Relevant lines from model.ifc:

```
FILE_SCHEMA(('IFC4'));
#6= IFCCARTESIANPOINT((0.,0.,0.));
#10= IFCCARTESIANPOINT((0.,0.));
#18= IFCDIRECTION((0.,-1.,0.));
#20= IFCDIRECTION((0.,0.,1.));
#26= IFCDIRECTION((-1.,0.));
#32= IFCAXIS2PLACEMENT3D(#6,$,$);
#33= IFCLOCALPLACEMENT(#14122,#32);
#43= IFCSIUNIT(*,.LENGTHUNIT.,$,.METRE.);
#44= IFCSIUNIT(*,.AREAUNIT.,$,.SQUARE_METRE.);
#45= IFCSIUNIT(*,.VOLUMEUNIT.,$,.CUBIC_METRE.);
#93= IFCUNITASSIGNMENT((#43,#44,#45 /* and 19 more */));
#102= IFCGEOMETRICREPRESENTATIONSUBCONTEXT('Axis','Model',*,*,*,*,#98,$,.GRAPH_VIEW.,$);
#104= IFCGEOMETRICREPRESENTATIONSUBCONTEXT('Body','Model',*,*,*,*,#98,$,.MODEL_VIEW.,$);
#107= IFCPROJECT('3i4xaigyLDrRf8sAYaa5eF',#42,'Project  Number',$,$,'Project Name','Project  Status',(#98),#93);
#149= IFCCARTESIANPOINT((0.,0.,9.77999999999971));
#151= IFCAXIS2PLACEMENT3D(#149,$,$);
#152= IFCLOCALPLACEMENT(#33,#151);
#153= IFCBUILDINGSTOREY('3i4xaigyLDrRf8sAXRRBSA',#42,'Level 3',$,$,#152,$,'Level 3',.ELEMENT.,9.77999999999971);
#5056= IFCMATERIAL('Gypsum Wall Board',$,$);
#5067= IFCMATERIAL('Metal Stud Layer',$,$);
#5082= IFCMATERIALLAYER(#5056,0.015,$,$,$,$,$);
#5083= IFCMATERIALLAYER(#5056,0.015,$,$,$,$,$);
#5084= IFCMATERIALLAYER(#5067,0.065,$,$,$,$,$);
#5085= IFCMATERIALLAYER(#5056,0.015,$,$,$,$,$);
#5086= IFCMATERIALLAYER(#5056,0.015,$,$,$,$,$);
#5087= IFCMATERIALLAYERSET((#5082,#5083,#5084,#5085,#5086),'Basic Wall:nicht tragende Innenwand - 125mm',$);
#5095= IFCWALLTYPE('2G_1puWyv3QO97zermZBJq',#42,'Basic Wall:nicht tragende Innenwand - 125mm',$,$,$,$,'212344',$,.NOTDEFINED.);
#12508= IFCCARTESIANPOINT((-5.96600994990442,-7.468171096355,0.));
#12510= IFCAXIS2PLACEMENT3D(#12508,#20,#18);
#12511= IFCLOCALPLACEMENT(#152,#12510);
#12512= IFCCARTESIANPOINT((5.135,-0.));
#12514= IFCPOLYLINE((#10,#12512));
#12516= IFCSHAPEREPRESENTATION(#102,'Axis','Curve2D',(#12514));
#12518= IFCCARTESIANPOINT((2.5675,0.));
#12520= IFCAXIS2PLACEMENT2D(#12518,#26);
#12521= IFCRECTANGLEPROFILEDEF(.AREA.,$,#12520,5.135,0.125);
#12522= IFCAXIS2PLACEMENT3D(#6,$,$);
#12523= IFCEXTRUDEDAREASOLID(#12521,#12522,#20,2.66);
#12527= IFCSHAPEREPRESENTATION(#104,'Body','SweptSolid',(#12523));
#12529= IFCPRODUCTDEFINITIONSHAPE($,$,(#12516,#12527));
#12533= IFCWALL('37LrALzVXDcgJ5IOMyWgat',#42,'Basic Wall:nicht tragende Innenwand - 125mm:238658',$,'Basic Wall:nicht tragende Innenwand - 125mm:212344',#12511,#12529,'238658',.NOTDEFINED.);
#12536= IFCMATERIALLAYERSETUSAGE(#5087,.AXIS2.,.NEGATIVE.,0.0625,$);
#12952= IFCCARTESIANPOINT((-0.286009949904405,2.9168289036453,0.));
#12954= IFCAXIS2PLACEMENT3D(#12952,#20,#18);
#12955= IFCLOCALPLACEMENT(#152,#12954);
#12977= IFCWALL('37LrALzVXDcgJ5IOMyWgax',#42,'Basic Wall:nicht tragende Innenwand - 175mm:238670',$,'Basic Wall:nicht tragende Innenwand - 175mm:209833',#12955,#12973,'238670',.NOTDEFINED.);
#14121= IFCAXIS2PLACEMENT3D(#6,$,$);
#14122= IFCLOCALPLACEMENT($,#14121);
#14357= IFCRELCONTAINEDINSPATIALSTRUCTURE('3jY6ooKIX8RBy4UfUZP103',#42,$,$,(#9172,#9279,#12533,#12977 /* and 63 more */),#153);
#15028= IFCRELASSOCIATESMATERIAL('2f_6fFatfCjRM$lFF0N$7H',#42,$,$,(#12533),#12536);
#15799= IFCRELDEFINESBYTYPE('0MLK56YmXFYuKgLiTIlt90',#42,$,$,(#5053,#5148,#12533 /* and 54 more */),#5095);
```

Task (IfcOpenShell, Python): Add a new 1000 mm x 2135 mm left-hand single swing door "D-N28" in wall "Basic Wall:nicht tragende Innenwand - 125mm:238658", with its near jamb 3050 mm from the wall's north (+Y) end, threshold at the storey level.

```python
import numpy as np
import ifcopenshell
import ifcopenshell.api.feature
import ifcopenshell.api.geometry
import ifcopenshell.api.root
import ifcopenshell.api.spatial
import ifcopenshell.geom
import ifcopenshell.util.element
import ifcopenshell.util.placement
import ifcopenshell.util.representation
import ifcopenshell.util.shape
import ifcopenshell.util.unit

model = ifcopenshell.open("model.ifc")
unit_scale = ifcopenshell.util.unit.calculate_unit_scale(model)
settings = ifcopenshell.geom.settings()


def volume(element):
    """Net volume in cubic metres, openings subtracted."""
    shape = ifcopenshell.geom.create_shape(settings, element)
    return ifcopenshell.util.shape.get_volume(shape.geometry)


wall = model.by_id(12533)
storey = ifcopenshell.util.element.get_container(wall, ifc_class="IfcBuildingStorey")
context = ifcopenshell.util.representation.get_context(model, "Model", "Body", "MODEL_VIEW")
before = volume(wall)

width, height, from_end, sill = 1, 2.135, 3.05, 0.0  # metres

# The wall runs along its own X axis, and the end named is its -X end.
wall_shape = ifcopenshell.geom.create_shape(settings, wall)
x, y, z = ifcopenshell.util.shape.get_vertices(wall_shape.geometry).T
start = x.min() + from_end
face, thickness = float(y.min()), float(y.max() - y.min())
wall_matrix = ifcopenshell.util.placement.get_local_placement(wall.ObjectPlacement)
level = ifcopenshell.util.placement.get_local_placement(storey.ObjectPlacement)[2, 3]


def in_wall(x, y):
    """Placement at x, y metres in the wall's axes, at sill height."""
    matrix = wall_matrix.copy()
    matrix[:, 3] = wall_matrix @ np.array([x / unit_scale, y / unit_scale, 0.0, 1.0])
    matrix[2, 3] = level + sill / unit_scale
    return matrix


# Opening: a box that overshoots both wall faces by 50 mm.
opening = ifcopenshell.api.root.create_entity(model, ifc_class="IfcOpeningElement", predefined_type="OPENING")
box = ifcopenshell.api.geometry.add_wall_representation(
    model, context=context, length=width, height=height, thickness=thickness + 0.1
)
ifcopenshell.api.geometry.assign_representation(model, product=opening, representation=box)
ifcopenshell.api.geometry.edit_object_placement(model, product=opening, matrix=in_wall(start, face - 0.05), is_si=False)
ifcopenshell.api.feature.add_feature(model, feature=opening, element=wall)

door = ifcopenshell.api.root.create_entity(model, ifc_class="IfcDoor", name="D-N28", predefined_type="DOOR")
door.OverallWidth, door.OverallHeight = width / unit_scale, height / unit_scale
door.OperationType = "SINGLE_SWING_LEFT"
body = ifcopenshell.api.geometry.add_door_representation(
    model,
    context=context,
    overall_width=door.OverallWidth,
    overall_height=door.OverallHeight,
    operation_type="SINGLE_SWING_LEFT",
    lining_properties={"LiningDepth": thickness / unit_scale, "ThresholdDepth": thickness / unit_scale},
)
ifcopenshell.api.geometry.assign_representation(model, product=door, representation=body)
ifcopenshell.api.spatial.assign_container(model, products=[door], relating_structure=storey)
ifcopenshell.api.feature.add_filling(model, opening=opening, element=door)

# The lining spans the wall, so the door starts at the wall face.
ifcopenshell.api.geometry.edit_object_placement(model, product=door, matrix=in_wall(start, face), is_si=False)

after = volume(wall)

print(f"wall volume {before:.3f} -> {after:.3f} m3")

model.write("model_rev.ifc")
```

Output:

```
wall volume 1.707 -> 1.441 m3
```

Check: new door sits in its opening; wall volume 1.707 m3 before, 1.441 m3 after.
